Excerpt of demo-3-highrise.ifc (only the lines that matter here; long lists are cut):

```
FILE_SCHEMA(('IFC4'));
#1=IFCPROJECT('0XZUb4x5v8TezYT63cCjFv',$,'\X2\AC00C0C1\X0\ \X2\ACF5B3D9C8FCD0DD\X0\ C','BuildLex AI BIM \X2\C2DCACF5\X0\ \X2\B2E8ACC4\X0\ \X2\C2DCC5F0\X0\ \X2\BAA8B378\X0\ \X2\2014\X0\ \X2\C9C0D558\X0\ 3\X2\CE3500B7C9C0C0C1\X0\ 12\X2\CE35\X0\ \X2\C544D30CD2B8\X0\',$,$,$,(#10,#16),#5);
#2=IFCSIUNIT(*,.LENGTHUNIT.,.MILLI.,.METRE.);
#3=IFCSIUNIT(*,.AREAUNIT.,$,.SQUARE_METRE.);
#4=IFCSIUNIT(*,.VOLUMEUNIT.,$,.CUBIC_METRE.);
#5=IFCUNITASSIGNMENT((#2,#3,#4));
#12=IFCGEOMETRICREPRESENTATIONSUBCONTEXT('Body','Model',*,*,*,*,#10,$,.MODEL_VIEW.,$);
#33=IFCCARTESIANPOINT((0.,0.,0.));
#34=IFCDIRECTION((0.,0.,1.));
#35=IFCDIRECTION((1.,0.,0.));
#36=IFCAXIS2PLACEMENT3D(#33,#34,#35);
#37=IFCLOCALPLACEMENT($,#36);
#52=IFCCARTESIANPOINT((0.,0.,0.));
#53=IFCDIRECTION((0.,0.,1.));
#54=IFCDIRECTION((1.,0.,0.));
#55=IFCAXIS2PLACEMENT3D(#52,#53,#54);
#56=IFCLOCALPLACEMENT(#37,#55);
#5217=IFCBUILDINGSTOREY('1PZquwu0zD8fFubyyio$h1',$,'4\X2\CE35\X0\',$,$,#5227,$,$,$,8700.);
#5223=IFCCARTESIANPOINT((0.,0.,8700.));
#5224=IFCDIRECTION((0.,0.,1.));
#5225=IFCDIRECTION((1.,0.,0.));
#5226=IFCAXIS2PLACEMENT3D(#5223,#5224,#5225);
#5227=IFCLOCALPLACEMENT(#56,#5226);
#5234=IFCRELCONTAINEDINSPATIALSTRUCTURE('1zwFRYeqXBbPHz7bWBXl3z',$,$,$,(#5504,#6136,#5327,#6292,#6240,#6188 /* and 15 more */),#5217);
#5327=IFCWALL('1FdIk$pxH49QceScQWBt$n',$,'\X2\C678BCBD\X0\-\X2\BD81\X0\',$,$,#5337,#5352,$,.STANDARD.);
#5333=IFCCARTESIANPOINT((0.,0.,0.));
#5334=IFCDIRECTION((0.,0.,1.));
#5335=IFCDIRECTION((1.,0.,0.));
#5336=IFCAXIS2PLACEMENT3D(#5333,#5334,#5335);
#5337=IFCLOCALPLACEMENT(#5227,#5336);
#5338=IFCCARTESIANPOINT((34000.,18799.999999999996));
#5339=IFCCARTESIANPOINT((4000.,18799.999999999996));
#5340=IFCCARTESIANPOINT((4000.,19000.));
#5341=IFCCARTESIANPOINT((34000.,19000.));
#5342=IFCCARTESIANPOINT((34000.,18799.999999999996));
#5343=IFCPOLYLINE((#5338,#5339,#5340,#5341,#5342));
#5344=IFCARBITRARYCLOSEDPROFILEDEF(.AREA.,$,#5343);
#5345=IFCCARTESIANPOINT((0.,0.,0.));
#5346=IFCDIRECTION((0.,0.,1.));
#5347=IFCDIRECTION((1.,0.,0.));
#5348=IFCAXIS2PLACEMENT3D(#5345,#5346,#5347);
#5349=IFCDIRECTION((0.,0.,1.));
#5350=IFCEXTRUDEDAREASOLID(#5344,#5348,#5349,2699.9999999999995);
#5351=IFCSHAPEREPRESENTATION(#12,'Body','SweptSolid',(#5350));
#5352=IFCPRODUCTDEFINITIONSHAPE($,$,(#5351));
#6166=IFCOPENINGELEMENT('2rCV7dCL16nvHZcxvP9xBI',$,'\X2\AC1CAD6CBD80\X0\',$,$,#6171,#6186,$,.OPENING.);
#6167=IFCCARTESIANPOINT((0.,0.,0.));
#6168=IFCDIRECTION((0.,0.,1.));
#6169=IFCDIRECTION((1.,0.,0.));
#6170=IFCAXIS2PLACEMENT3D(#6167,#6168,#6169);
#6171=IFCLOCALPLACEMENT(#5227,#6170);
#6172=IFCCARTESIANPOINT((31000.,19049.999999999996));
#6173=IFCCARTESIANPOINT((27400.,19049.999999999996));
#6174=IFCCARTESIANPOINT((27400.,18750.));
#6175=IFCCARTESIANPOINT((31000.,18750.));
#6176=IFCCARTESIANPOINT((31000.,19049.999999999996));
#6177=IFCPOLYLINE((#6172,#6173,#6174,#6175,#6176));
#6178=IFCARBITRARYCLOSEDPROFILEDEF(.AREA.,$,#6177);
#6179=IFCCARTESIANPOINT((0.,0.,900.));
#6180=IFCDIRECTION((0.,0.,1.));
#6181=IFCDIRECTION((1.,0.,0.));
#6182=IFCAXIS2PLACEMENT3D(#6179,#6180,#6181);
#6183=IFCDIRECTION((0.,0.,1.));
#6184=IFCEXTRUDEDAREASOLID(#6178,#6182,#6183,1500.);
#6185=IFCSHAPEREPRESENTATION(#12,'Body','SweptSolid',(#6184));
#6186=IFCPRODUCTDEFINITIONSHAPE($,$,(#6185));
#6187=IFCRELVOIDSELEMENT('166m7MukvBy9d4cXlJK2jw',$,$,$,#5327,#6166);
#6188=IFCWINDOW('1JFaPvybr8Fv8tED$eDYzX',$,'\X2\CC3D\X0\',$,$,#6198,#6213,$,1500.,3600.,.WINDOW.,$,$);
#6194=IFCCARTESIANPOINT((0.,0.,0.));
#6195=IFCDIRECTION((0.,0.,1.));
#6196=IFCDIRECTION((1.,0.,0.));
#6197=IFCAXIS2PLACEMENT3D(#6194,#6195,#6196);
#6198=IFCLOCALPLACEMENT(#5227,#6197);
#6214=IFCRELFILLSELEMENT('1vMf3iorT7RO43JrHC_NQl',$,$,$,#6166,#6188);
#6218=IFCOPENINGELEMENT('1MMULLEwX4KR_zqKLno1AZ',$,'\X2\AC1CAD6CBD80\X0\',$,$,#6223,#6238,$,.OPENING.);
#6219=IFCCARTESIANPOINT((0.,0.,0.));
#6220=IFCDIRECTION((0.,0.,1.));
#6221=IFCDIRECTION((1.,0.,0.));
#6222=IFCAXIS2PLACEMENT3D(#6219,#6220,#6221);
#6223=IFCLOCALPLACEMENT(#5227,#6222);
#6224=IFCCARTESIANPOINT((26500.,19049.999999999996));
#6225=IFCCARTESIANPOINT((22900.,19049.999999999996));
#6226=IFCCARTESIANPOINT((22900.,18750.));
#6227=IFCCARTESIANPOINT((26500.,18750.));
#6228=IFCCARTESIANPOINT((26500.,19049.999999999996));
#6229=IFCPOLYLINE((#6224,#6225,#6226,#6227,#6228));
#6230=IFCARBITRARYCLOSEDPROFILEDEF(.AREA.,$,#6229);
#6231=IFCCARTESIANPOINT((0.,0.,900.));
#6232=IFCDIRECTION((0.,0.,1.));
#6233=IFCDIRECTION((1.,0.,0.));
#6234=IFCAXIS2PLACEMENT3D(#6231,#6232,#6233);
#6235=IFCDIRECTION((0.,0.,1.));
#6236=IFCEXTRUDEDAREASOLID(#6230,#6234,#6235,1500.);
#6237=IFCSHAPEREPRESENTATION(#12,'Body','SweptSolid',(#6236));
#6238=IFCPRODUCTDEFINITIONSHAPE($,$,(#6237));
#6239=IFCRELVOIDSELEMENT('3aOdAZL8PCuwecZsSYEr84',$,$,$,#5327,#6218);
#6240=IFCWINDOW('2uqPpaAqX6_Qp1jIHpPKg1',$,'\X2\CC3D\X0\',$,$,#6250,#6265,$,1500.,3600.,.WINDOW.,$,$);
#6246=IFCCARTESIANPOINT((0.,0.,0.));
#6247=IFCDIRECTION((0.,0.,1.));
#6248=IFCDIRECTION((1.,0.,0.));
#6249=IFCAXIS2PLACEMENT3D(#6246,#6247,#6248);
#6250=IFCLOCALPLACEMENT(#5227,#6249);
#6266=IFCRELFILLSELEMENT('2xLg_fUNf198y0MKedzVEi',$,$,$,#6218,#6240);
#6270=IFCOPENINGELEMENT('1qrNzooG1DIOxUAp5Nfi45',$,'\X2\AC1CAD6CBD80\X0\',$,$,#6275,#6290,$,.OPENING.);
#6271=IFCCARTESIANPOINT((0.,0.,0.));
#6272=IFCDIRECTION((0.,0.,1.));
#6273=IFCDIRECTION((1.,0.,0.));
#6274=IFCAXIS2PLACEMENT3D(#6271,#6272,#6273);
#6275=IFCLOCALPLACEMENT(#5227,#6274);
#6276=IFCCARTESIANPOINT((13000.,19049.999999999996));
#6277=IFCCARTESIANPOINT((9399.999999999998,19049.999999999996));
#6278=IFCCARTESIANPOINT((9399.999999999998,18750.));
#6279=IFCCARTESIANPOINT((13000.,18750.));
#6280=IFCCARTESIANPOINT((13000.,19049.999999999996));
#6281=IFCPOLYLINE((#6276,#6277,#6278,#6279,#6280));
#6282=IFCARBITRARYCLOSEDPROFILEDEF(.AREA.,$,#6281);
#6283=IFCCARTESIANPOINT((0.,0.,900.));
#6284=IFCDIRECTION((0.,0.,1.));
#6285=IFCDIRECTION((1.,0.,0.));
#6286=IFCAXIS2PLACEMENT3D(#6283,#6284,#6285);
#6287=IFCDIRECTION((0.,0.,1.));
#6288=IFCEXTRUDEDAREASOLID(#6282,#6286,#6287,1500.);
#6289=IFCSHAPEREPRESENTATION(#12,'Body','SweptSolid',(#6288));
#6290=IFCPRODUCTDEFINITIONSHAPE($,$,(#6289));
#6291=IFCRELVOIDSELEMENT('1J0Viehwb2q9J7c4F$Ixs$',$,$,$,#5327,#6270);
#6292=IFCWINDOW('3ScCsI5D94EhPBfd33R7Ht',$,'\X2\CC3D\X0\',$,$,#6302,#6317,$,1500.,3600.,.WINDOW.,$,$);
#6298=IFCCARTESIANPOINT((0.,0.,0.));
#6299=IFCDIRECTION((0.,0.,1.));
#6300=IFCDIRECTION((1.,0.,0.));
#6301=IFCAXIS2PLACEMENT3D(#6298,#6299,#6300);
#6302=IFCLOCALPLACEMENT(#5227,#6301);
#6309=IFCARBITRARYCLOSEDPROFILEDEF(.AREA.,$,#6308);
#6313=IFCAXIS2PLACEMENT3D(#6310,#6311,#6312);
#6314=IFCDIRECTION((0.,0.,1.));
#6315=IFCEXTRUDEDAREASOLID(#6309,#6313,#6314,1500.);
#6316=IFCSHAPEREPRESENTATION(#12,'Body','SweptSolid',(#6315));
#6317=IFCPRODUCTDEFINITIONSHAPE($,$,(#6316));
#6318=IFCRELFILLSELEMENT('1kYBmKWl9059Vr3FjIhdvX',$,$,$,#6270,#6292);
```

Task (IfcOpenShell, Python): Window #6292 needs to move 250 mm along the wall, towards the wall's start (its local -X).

```python
import ifcopenshell
import ifcopenshell.api.geometry
import ifcopenshell.util.placement
import ifcopenshell.util.unit

model = ifcopenshell.open("demo-3-highrise.ifc")
unit_scale = ifcopenshell.util.unit.calculate_unit_scale(model)

window = model.by_guid("3ScCsI5D94EhPBfd33R7Ht")
opening = window.FillsVoids[0].RelatingOpeningElement
wall = opening.VoidsElements[0].RelatingBuildingElement

wall_matrix = ifcopenshell.util.placement.get_local_placement(wall.ObjectPlacement)
shift = wall_matrix[:3, 0] * -0.25 / unit_scale
before = ifcopenshell.util.placement.get_local_placement(window.ObjectPlacement)[:3, 3].copy()

# The window is not placed relative to its opening, so move both.
for product in (opening, window):
    matrix = ifcopenshell.util.placement.get_local_placement(product.ObjectPlacement)
    matrix[:3, 3] += shift
    ifcopenshell.api.geometry.edit_object_placement(model, product=product, matrix=matrix, is_si=False)

after = ifcopenshell.util.placement.get_local_placement(window.ObjectPlacement)[:3, 3]
print("window moved by", (after - before).round(3) + 0.0)

model.write("demo-3-highrise-out.ifc")
```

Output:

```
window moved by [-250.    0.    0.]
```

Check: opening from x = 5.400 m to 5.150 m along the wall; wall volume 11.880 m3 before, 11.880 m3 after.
